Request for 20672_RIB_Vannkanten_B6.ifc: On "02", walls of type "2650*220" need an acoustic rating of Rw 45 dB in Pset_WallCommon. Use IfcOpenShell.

First a look at what the model holds.

```python
import ifcopenshell
import ifcopenshell.util.element

model = ifcopenshell.open("20672_RIB_Vannkanten_B6.ifc")
print(model.schema)
storey = next(s for s in model.by_type("IfcBuildingStorey") if s.Name == "02")
walls = [e for e in ifcopenshell.util.element.get_decomposition(storey) if e.is_a("IfcWall")]
seen = {}
for e in walls:
    element_type = ifcopenshell.util.element.get_type(e)
    key = (element_type.Name if element_type != e and element_type else None, ifcopenshell.util.element.get_pset(e, "Pset_WallCommon", "AcousticRating"))
    seen[key] = seen.get(key, 0) + 1
for (name, value), count in sorted(seen.items(), key=str):
    print(count, "x", name, "|", value)
```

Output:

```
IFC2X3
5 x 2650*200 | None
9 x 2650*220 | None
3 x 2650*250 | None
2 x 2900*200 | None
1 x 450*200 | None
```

```python
import ifcopenshell
import ifcopenshell.api.pset
import ifcopenshell.util.element

model = ifcopenshell.open("20672_RIB_Vannkanten_B6.ifc")

storey = next(s for s in model.by_type("IfcBuildingStorey") if s.Name == "02")
walls = [e for e in ifcopenshell.util.element.get_decomposition(storey) if e.is_a("IfcWall")]

count = 0
for e in walls:
    element_type = ifcopenshell.util.element.get_type(e)
    if element_type in (None, e) or element_type.Name != "2650*220":
        continue
    # add_pset returns the element's existing set when there is one.
    pset = ifcopenshell.api.pset.add_pset(model, product=e, name="Pset_WallCommon")
    ifcopenshell.api.pset.edit_pset(model, pset=pset, properties={"AcousticRating": "Rw 45 dB"})
    count += 1

print(count, "walls updated")

model.write("20672_RIB_Vannkanten_B6_rev.ifc")
```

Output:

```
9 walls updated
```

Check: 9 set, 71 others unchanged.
